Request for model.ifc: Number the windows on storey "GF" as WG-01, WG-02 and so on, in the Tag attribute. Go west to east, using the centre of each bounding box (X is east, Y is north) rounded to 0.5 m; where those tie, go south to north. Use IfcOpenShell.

First a look at what the model holds.

```python
import ifcopenshell
import ifcopenshell.util.element
import ifcopenshell.util.placement

model = ifcopenshell.open("model.ifc")
print(model.schema)
storey = next(s for s in model.by_type("IfcBuildingStorey") if s.Name == "GF")
windows = [e for e in ifcopenshell.util.element.get_decomposition(storey) if e.is_a("IfcWindow")]
for e in sorted(windows, key=lambda e: e.id()):
    origin = ifcopenshell.util.placement.get_local_placement(e.ObjectPlacement)[:3, 3]
    print(e.id(), e.Tag, e.Name, origin.round(2) + 0.0, sep=" | ")
```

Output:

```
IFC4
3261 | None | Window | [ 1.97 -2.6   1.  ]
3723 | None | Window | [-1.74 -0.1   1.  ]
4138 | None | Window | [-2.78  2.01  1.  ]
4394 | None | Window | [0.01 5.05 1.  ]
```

```python
import ifcopenshell
import ifcopenshell.geom
import ifcopenshell.util.element
import ifcopenshell.util.shape

model = ifcopenshell.open("model.ifc")
settings = ifcopenshell.geom.settings()
settings.set("use-world-coords", True)


def centre(element):
    shape = ifcopenshell.geom.create_shape(settings, element)
    return ifcopenshell.util.shape.get_bbox_centroid(shape.geometry)


storey = next(s for s in model.by_type("IfcBuildingStorey") if s.Name == "GF")
windows = [e for e in ifcopenshell.util.element.get_decomposition(storey) if e.is_a("IfcWindow")]

# Insertion points can sit at a corner or the storey origin, so sort by the geometry (in metres).
centres = {e: centre(e) for e in windows}
windows.sort(key=lambda e: (round(centres[e][0] / 0.5), centres[e][1]))

for i, e in enumerate(windows, start=1):
    number = f"WG-{i:02d}"
    e.Tag = number
    print(e.id(), number)

model.write("model-out.ifc")
```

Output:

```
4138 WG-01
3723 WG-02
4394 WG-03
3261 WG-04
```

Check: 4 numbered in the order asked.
